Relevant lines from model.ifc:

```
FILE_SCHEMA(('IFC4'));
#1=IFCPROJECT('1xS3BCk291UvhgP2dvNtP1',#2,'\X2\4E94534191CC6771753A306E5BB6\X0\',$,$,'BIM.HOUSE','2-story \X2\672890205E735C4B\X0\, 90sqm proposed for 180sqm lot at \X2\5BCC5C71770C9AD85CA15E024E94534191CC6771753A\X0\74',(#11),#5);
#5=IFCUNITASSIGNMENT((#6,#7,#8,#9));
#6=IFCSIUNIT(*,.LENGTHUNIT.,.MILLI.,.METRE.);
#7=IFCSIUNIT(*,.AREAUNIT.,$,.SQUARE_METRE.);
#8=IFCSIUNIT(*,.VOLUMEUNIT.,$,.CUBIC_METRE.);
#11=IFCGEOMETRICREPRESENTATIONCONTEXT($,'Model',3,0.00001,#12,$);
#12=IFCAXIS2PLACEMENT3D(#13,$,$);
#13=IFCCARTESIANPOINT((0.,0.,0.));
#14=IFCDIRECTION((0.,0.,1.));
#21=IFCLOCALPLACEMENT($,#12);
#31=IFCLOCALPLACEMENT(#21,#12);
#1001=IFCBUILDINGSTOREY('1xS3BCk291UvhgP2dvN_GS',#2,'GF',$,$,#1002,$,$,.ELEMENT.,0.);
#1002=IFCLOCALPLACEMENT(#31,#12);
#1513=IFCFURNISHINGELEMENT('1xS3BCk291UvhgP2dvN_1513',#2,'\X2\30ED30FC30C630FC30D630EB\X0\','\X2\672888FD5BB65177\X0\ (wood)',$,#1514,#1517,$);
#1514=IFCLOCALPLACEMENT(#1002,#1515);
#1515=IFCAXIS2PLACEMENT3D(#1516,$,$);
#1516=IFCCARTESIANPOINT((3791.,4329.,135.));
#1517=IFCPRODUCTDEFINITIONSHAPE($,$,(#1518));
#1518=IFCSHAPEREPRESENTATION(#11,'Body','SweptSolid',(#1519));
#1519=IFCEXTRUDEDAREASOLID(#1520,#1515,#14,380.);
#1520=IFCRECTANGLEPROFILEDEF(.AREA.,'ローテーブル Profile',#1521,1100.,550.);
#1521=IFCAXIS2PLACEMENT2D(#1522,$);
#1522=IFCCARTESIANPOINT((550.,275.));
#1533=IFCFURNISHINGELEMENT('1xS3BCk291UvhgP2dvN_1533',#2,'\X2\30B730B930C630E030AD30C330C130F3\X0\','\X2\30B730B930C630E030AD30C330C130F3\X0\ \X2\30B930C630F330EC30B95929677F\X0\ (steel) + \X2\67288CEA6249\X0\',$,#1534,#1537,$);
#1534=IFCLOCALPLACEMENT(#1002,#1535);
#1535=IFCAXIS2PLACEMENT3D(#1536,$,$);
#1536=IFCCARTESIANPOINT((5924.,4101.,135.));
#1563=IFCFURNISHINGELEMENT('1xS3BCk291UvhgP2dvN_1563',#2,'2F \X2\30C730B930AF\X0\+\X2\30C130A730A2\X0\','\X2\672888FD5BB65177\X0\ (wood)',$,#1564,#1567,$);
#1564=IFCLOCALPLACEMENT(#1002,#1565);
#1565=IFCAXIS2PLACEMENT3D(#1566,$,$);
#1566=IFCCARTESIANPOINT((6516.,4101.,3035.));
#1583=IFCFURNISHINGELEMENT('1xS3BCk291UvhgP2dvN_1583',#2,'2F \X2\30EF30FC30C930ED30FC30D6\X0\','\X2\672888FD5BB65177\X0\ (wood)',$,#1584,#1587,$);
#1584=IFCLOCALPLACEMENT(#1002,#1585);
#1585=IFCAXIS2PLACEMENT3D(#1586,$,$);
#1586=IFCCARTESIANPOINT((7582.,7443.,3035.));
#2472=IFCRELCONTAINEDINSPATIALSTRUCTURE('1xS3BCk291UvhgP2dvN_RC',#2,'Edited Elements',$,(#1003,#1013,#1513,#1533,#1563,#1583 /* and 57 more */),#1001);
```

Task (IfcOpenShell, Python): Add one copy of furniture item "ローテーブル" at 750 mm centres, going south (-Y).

```python
import numpy as np
import ifcopenshell
import ifcopenshell.api.geometry
import ifcopenshell.api.root
import ifcopenshell.util.element
import ifcopenshell.util.placement

model = ifcopenshell.open("model.ifc")


def reuse_history(source, copy):
    """copy_class also copies each property set's owner history, people and application; keep the originals."""
    for rel in copy.IsDefinedBy:
        if rel.is_a("IfcRelDefinesByProperties") and (history := rel.RelatingPropertyDefinition.OwnerHistory):
            rel.RelatingPropertyDefinition.OwnerHistory = source.OwnerHistory
            ifcopenshell.util.element.remove_deep2(model, history)


source = model.by_guid("1xS3BCk291UvhgP2dvN_1513")
base = ifcopenshell.util.placement.get_local_placement(source.ObjectPlacement)
step = np.array([0.0, -1.0, 0.0]) * 750.0

for i in range(1, 2):
    copy = ifcopenshell.api.root.copy_class(model, product=source)
    copy.Representation = ifcopenshell.util.element.copy_deep(
        model, source.Representation, exclude=["IfcGeometricRepresentationContext", "IfcRepresentationMap"]
    )
    reuse_history(source, copy)
    matrix = base.copy()
    matrix[:3, 3] += i * step
    print("added at", matrix[:3, 3].round(3) + 0.0)
    ifcopenshell.api.geometry.edit_object_placement(model, product=copy, matrix=matrix, is_si=False)

model.write("model_updated.ifc")
```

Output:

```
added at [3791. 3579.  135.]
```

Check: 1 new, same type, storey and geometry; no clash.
